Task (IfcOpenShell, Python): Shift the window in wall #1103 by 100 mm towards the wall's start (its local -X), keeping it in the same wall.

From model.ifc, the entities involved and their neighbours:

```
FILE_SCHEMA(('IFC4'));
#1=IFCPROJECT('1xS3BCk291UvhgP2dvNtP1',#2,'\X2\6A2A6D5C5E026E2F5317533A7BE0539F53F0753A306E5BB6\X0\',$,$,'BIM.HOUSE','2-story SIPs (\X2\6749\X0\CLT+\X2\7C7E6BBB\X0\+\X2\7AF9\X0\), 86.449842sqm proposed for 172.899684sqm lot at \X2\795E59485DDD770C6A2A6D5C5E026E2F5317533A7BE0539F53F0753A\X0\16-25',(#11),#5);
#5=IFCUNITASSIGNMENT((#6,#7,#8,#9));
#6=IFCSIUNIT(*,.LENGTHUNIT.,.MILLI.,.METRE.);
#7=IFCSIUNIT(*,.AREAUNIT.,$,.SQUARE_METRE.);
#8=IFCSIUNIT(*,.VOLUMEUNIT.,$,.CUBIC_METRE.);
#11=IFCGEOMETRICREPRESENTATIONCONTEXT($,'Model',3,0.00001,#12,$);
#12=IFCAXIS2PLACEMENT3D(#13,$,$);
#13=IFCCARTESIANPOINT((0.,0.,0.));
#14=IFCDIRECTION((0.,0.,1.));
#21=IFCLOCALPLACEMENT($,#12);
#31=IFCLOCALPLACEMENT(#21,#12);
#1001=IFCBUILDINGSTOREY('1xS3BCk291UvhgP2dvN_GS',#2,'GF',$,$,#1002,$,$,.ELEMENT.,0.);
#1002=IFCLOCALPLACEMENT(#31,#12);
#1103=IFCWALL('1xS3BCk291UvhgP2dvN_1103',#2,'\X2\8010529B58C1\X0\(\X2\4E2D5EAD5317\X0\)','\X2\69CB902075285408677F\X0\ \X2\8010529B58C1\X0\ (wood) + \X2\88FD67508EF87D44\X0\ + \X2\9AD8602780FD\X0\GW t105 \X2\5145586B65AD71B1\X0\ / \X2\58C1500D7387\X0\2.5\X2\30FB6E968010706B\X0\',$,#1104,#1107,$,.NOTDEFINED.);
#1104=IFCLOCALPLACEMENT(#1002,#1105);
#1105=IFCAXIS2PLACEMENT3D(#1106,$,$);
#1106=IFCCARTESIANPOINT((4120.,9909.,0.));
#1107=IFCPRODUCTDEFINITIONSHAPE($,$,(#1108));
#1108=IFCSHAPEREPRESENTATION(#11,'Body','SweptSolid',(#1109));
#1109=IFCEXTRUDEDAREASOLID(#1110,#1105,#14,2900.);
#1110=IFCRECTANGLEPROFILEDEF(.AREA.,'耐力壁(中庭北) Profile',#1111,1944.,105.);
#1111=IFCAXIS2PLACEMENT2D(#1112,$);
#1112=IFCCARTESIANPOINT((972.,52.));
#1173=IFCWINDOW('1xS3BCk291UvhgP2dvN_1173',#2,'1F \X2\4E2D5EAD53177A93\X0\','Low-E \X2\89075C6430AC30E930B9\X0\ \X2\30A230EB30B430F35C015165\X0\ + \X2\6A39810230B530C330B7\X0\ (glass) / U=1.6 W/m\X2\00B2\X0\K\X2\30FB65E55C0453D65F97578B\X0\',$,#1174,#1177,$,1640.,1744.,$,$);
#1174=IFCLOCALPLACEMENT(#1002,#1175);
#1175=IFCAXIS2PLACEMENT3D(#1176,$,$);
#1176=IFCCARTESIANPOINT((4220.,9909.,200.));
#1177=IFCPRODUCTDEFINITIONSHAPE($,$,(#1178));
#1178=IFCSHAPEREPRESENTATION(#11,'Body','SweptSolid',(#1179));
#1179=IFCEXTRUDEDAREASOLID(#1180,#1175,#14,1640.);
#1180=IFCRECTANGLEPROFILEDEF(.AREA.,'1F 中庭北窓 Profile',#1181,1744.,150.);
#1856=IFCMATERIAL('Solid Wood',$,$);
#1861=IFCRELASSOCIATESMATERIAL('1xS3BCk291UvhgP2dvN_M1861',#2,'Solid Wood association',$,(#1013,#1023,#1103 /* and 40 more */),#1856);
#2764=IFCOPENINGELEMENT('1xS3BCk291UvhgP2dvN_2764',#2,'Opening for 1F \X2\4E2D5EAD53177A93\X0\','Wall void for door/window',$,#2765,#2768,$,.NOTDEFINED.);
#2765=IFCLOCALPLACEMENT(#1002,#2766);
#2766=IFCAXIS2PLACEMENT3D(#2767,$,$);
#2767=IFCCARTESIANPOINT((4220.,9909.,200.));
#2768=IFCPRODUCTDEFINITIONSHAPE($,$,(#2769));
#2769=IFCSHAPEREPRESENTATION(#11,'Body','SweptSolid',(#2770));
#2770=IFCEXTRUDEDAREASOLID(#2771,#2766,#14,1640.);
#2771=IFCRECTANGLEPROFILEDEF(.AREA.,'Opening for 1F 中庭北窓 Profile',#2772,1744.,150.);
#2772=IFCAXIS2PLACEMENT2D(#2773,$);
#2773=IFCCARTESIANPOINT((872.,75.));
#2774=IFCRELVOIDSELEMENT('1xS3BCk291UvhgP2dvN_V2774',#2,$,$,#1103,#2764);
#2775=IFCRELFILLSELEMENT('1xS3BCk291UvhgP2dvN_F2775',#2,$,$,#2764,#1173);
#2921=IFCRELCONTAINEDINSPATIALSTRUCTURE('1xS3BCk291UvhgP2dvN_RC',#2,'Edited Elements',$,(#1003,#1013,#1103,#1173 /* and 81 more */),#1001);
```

```python
import ifcopenshell
import ifcopenshell.api.geometry
import ifcopenshell.util.placement
import ifcopenshell.util.unit

model = ifcopenshell.open("model.ifc")
unit_scale = ifcopenshell.util.unit.calculate_unit_scale(model)

window = model.by_guid("1xS3BCk291UvhgP2dvN_1173")
opening = window.FillsVoids[0].RelatingOpeningElement
wall = opening.VoidsElements[0].RelatingBuildingElement

wall_matrix = ifcopenshell.util.placement.get_local_placement(wall.ObjectPlacement)
shift = wall_matrix[:3, 0] * -0.1 / unit_scale
before = ifcopenshell.util.placement.get_local_placement(window.ObjectPlacement)[:3, 3].copy()

# The window is not placed relative to its opening, so move both.
for product in (opening, window):
    matrix = ifcopenshell.util.placement.get_local_placement(product.ObjectPlacement)
    matrix[:3, 3] += shift
    ifcopenshell.api.geometry.edit_object_placement(model, product=product, matrix=matrix, is_si=False)

after = ifcopenshell.util.placement.get_local_placement(window.ObjectPlacement)[:3, 3]
print("window moved by", (after - before).round(3) + 0.0)

model.write("model_v2.ifc")
```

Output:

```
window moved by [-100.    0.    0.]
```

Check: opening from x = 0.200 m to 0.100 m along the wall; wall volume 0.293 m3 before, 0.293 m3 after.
